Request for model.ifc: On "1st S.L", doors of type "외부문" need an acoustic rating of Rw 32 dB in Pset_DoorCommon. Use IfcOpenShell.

First a look at what the model holds.

```python
import ifcopenshell
import ifcopenshell.util.element

model = ifcopenshell.open("model.ifc")
print(model.schema)
storey = next(s for s in model.by_type("IfcBuildingStorey") if s.Name == "1st S.L")
doors = [e for e in ifcopenshell.util.element.get_decomposition(storey) if e.is_a("IfcDoor")]
seen = {}
for e in doors:
    element_type = ifcopenshell.util.element.get_type(e)
    key = (element_type.Name if element_type != e and element_type else None, ifcopenshell.util.element.get_pset(e, "Pset_DoorCommon", "AcousticRating"))
    seen[key] = seen.get(key, 0) + 1
for (name, value), count in sorted(seen.items(), key=str):
    print(count, "x", name, "|", value)
```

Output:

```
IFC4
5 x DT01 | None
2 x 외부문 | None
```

```python
import ifcopenshell
import ifcopenshell.api.pset
import ifcopenshell.util.element

model = ifcopenshell.open("model.ifc")

storey = next(s for s in model.by_type("IfcBuildingStorey") if s.Name == "1st S.L")
doors = [e for e in ifcopenshell.util.element.get_decomposition(storey) if e.is_a("IfcDoor")]

count = 0
for e in doors:
    element_type = ifcopenshell.util.element.get_type(e)
    if element_type in (None, e) or element_type.Name != "외부문":
        continue
    # add_pset returns the element's existing set when there is one.
    pset = ifcopenshell.api.pset.add_pset(model, product=e, name="Pset_DoorCommon")
    ifcopenshell.api.pset.edit_pset(model, pset=pset, properties={"AcousticRating": "Rw 32 dB"})
    count += 1

print(count, "doors updated")

model.write("model_v2.ifc")
```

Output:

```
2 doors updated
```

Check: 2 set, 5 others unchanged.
